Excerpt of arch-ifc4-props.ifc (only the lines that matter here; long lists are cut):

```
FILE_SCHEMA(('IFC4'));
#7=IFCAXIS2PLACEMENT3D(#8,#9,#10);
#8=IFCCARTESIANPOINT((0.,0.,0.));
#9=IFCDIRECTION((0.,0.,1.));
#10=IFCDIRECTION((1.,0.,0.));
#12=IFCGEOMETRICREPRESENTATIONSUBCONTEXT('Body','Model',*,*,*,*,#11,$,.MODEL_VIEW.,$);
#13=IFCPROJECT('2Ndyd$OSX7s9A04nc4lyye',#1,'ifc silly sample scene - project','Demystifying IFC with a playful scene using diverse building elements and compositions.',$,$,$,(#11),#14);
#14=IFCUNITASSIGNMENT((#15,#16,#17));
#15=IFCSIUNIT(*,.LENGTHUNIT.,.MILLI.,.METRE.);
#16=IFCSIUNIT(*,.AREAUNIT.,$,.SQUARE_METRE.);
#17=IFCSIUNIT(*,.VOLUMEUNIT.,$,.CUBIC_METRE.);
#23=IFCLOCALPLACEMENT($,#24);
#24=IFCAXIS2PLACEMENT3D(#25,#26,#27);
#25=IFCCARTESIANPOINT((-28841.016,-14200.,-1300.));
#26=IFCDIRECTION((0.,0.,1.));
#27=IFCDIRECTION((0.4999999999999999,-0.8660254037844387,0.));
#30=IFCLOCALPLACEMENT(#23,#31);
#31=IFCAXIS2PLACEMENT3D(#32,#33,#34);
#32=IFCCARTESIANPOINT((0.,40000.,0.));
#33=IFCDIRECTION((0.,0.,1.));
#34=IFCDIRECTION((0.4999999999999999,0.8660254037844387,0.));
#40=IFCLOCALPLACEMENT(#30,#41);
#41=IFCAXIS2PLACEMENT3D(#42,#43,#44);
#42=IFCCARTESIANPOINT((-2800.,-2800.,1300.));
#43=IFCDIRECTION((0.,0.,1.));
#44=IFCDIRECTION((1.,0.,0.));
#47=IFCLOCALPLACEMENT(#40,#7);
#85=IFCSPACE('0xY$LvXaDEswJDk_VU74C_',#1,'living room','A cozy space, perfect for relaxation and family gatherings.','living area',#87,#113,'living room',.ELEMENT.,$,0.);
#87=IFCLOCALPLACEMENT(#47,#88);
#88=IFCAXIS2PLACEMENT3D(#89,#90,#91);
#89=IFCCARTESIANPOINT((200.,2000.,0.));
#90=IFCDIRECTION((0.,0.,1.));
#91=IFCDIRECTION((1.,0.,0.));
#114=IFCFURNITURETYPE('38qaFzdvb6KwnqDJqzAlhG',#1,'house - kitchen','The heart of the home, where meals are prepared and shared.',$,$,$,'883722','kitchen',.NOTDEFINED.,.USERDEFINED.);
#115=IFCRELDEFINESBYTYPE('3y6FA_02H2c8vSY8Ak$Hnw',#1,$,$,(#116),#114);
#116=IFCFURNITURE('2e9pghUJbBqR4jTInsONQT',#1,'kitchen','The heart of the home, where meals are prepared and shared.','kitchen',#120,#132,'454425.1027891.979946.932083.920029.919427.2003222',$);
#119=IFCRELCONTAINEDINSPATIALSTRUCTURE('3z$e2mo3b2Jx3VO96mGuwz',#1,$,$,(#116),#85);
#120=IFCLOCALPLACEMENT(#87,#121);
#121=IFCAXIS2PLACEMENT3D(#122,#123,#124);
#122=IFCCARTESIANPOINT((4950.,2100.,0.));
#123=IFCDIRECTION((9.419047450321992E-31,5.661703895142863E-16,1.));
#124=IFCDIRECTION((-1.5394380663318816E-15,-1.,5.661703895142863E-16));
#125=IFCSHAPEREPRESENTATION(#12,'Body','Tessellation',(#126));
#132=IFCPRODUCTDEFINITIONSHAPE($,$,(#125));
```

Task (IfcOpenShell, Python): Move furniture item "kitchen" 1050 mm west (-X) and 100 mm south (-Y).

```python
import ifcopenshell
import ifcopenshell.api.geometry
import ifcopenshell.util.placement
import ifcopenshell.util.unit

model = ifcopenshell.open("arch-ifc4-props.ifc")
unit_scale = ifcopenshell.util.unit.calculate_unit_scale(model)

item = model.by_guid("2e9pghUJbBqR4jTInsONQT")
matrix = ifcopenshell.util.placement.get_local_placement(item.ObjectPlacement)
matrix[0, 3] -= 1.05 / unit_scale
matrix[1, 3] -= 0.1 / unit_scale
ifcopenshell.api.geometry.edit_object_placement(model, product=item, matrix=matrix, is_si=False)

print(ifcopenshell.util.placement.get_local_placement(item.ObjectPlacement).round(3) + 0.0)

model.write("arch-ifc4-props_edited.ifc")
```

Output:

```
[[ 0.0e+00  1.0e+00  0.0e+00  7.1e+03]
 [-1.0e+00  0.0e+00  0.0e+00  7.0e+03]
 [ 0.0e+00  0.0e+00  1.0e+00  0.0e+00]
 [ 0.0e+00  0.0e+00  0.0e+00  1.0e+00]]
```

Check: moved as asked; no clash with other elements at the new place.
